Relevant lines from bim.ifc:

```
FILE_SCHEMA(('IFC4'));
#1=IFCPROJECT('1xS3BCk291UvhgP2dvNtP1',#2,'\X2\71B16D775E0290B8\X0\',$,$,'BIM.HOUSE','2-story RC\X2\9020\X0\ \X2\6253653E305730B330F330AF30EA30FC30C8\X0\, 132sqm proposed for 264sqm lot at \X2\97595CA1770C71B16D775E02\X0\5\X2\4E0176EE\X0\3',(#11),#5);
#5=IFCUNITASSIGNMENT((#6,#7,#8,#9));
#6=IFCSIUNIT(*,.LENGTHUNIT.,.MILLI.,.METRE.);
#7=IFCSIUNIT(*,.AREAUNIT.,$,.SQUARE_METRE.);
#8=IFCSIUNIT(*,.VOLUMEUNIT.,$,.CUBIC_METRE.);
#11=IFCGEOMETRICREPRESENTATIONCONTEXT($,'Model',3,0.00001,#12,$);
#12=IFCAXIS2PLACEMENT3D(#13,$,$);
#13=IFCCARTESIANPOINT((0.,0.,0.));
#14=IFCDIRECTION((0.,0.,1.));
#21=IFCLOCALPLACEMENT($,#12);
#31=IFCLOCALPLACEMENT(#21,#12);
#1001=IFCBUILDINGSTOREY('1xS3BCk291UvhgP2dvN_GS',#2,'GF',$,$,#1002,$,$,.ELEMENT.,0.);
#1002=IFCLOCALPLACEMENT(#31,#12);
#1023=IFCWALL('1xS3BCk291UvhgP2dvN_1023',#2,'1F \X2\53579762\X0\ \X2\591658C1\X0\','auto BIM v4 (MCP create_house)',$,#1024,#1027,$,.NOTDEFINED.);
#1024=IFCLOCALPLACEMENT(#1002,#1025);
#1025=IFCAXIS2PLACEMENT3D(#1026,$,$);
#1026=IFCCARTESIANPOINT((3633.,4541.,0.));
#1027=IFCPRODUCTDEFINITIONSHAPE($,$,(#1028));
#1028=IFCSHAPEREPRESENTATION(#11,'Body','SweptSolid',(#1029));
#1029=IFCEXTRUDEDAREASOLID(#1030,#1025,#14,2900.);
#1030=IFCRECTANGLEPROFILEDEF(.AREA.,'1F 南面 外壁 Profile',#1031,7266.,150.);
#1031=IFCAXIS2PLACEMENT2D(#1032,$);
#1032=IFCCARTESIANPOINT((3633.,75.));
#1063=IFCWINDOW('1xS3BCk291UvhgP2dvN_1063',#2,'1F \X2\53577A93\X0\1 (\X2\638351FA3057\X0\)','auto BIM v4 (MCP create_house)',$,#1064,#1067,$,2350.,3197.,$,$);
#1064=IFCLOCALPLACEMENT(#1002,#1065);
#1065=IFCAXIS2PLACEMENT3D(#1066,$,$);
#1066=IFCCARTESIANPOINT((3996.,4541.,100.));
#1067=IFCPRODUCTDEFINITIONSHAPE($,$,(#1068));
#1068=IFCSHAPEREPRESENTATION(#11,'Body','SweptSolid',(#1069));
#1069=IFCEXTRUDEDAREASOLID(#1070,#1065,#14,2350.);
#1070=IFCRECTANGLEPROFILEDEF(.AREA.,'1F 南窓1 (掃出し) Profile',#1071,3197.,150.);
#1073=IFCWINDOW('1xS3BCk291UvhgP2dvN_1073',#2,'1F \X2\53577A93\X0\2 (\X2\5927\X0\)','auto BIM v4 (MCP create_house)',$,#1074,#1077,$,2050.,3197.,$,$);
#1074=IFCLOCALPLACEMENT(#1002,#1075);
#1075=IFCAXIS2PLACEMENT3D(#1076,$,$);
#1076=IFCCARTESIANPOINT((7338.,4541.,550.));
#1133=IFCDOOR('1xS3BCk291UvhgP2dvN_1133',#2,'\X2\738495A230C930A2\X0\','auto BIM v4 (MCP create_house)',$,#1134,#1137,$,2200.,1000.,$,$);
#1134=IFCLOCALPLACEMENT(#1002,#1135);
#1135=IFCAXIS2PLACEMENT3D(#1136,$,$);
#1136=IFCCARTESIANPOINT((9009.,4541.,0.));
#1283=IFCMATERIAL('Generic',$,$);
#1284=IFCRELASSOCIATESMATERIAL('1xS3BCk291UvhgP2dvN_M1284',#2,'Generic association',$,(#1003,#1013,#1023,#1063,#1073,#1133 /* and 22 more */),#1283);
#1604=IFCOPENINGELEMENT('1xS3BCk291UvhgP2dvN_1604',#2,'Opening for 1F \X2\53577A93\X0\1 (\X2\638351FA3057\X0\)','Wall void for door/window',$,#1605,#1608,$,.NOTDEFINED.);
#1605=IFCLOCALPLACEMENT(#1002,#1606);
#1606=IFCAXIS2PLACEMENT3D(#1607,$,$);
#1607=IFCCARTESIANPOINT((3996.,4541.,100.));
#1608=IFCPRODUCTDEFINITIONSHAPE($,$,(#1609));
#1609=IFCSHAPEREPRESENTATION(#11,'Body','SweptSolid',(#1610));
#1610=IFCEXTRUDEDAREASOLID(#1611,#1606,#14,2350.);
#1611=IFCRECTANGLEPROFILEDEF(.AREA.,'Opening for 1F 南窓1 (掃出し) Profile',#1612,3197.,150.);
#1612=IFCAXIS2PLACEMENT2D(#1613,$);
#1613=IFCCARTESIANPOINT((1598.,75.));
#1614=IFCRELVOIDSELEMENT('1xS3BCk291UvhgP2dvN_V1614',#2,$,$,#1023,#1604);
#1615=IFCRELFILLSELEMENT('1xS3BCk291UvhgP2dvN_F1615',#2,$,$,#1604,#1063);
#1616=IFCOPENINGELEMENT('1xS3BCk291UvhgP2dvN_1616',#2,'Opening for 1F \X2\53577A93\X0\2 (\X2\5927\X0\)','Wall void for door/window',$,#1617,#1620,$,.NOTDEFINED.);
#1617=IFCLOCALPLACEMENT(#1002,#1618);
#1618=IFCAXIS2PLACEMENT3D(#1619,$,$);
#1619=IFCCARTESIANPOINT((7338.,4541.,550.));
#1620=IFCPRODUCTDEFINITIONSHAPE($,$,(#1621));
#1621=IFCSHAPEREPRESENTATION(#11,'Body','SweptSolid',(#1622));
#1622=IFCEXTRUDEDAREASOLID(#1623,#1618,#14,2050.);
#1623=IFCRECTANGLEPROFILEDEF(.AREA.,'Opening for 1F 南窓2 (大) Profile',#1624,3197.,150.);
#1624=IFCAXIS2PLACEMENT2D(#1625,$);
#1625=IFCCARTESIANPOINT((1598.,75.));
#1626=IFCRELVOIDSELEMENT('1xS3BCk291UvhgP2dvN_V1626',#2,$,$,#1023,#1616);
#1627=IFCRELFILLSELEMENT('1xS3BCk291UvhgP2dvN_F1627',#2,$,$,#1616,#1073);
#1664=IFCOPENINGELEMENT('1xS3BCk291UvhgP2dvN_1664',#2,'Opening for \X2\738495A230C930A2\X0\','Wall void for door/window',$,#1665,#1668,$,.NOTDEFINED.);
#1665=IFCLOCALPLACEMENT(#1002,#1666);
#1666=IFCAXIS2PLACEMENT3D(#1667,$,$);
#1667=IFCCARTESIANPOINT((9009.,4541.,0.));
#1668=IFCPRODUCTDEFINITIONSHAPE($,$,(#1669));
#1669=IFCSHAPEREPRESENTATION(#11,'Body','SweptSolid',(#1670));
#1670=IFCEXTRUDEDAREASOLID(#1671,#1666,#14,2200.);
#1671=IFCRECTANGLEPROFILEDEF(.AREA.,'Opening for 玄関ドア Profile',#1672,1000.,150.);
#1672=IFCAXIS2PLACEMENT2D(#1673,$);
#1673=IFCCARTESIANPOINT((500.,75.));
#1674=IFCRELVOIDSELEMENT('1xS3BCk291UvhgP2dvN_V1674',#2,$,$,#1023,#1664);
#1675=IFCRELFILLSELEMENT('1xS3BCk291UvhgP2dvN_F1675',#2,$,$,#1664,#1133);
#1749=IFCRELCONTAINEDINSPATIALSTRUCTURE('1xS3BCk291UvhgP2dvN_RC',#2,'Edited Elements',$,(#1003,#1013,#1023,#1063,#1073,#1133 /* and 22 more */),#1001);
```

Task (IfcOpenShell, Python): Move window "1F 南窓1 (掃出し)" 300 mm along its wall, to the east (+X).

```python
import ifcopenshell
import ifcopenshell.api.geometry
import ifcopenshell.util.placement
import ifcopenshell.util.unit

model = ifcopenshell.open("bim.ifc")
unit_scale = ifcopenshell.util.unit.calculate_unit_scale(model)

window = model.by_guid("1xS3BCk291UvhgP2dvN_1063")
opening = window.FillsVoids[0].RelatingOpeningElement
wall = opening.VoidsElements[0].RelatingBuildingElement

wall_matrix = ifcopenshell.util.placement.get_local_placement(wall.ObjectPlacement)
shift = wall_matrix[:3, 0] * 0.3 / unit_scale
before = ifcopenshell.util.placement.get_local_placement(window.ObjectPlacement)[:3, 3].copy()

# The window is not placed relative to its opening, so move both.
for product in (opening, window):
    matrix = ifcopenshell.util.placement.get_local_placement(product.ObjectPlacement)
    matrix[:3, 3] += shift
    ifcopenshell.api.geometry.edit_object_placement(model, product=product, matrix=matrix, is_si=False)

after = ifcopenshell.util.placement.get_local_placement(window.ObjectPlacement)[:3, 3]
print("window moved by", (after - before).round(3) + 0.0)

model.write("bim_updated.ifc")
```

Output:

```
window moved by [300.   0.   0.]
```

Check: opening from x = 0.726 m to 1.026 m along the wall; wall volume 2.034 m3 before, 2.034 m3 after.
